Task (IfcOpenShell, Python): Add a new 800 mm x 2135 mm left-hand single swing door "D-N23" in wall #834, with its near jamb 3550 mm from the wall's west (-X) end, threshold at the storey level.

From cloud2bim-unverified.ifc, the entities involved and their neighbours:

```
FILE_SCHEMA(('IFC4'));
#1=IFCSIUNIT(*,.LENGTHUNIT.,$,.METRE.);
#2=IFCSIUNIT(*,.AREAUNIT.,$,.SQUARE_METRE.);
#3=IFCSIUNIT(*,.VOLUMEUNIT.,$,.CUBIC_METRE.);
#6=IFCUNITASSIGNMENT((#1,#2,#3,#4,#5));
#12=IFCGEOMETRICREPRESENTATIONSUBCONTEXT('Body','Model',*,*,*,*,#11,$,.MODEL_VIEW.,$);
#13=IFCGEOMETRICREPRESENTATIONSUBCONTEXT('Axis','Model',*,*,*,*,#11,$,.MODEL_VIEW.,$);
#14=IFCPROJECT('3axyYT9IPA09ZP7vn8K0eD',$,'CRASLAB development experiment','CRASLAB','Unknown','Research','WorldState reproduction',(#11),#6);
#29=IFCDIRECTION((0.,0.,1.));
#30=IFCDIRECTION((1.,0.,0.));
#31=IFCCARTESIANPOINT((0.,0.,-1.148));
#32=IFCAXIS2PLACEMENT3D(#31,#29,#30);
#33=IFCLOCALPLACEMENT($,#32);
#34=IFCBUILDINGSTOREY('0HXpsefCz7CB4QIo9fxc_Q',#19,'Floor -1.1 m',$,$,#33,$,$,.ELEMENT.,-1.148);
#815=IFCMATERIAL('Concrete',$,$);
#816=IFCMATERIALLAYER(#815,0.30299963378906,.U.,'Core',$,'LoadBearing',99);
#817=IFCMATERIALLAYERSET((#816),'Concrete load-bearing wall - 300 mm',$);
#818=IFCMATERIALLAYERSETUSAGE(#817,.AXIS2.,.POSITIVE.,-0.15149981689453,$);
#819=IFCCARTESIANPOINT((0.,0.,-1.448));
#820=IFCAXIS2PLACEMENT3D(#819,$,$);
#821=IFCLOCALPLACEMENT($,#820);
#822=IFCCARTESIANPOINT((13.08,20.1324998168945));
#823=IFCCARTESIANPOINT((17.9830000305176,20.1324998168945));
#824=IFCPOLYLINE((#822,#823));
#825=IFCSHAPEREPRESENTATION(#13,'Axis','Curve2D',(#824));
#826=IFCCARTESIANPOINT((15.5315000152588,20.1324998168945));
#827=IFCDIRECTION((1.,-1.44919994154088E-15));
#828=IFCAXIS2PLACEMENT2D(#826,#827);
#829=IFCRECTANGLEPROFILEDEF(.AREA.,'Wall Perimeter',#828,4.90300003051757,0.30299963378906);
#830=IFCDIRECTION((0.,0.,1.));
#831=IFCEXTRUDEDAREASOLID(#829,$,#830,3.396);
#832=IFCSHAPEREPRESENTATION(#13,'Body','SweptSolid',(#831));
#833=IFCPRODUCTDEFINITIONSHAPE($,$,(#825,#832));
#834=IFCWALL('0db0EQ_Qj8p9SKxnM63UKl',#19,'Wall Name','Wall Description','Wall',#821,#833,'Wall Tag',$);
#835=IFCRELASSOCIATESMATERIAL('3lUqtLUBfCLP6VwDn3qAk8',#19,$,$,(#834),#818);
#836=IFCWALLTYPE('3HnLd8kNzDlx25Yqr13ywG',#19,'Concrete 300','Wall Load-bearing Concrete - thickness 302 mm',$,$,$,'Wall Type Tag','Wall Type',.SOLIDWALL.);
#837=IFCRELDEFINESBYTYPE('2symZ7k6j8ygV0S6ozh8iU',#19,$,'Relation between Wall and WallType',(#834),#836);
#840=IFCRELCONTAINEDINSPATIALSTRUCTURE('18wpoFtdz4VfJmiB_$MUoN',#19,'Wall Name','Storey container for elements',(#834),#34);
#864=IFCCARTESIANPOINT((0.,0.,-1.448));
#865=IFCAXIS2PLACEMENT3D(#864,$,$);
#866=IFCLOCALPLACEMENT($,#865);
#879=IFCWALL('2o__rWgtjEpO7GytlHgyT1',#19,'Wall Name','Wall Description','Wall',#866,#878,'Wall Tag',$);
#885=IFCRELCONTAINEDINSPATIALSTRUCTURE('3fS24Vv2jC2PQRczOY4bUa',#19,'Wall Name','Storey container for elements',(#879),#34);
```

```python
import numpy as np
import ifcopenshell
import ifcopenshell.api.feature
import ifcopenshell.api.geometry
import ifcopenshell.api.root
import ifcopenshell.api.spatial
import ifcopenshell.geom
import ifcopenshell.util.element
import ifcopenshell.util.placement
import ifcopenshell.util.representation
import ifcopenshell.util.shape
import ifcopenshell.util.unit

model = ifcopenshell.open("cloud2bim-unverified.ifc")
unit_scale = ifcopenshell.util.unit.calculate_unit_scale(model)
settings = ifcopenshell.geom.settings()


def volume(element):
    """Net volume in cubic metres, openings subtracted."""
    shape = ifcopenshell.geom.create_shape(settings, element)
    return ifcopenshell.util.shape.get_volume(shape.geometry)


wall = model.by_guid("0db0EQ_Qj8p9SKxnM63UKl")
storey = ifcopenshell.util.element.get_container(wall, ifc_class="IfcBuildingStorey")
context = ifcopenshell.util.representation.get_context(model, "Model", "Body", "MODEL_VIEW")
before = volume(wall)

width, height, from_end, sill = 0.8, 2.135, 3.55, 0.0  # metres

# The wall runs along its own X axis, and the end named is its -X end.
wall_shape = ifcopenshell.geom.create_shape(settings, wall)
x, y, z = ifcopenshell.util.shape.get_vertices(wall_shape.geometry).T
start = x.min() + from_end
face, thickness = float(y.min()), float(y.max() - y.min())
wall_matrix = ifcopenshell.util.placement.get_local_placement(wall.ObjectPlacement)
level = ifcopenshell.util.placement.get_local_placement(storey.ObjectPlacement)[2, 3]


def in_wall(x, y):
    """Placement at x, y metres in the wall's axes, at sill height."""
    matrix = wall_matrix.copy()
    matrix[:, 3] = wall_matrix @ np.array([x / unit_scale, y / unit_scale, 0.0, 1.0])
    matrix[2, 3] = level + sill / unit_scale
    return matrix


# Opening: a box that overshoots both wall faces by 50 mm.
opening = ifcopenshell.api.root.create_entity(model, ifc_class="IfcOpeningElement", predefined_type="OPENING")
box = ifcopenshell.api.geometry.add_wall_representation(
    model, context=context, length=width, height=height, thickness=thickness + 0.1
)
ifcopenshell.api.geometry.assign_representation(model, product=opening, representation=box)
ifcopenshell.api.geometry.edit_object_placement(model, product=opening, matrix=in_wall(start, face - 0.05), is_si=False)
ifcopenshell.api.feature.add_feature(model, feature=opening, element=wall)

door = ifcopenshell.api.root.create_entity(model, ifc_class="IfcDoor", name="D-N23", predefined_type="DOOR")
door.OverallWidth, door.OverallHeight = width / unit_scale, height / unit_scale
door.OperationType = "SINGLE_SWING_LEFT"
body = ifcopenshell.api.geometry.add_door_representation(
    model,
    context=context,
    overall_width=door.OverallWidth,
    overall_height=door.OverallHeight,
    operation_type="SINGLE_SWING_LEFT",
    lining_properties={"LiningDepth": thickness / unit_scale, "ThresholdDepth": thickness / unit_scale},
)
ifcopenshell.api.geometry.assign_representation(model, product=door, representation=body)
ifcopenshell.api.spatial.assign_container(model, products=[door], relating_structure=storey)
ifcopenshell.api.feature.add_filling(model, opening=opening, element=door)

# The lining spans the wall, so the door starts at the wall face.
ifcopenshell.api.geometry.edit_object_placement(model, product=door, matrix=in_wall(start, face), is_si=False)

after = volume(wall)

print(f"wall volume {before:.3f} -> {after:.3f} m3")

model.write("cloud2bim-unverified_updated.ifc")
```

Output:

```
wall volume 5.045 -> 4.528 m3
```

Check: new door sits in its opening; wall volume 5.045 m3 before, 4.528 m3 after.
